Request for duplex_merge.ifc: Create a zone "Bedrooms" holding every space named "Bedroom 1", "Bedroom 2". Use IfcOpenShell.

First a look at what the model holds.

```python
import ifcopenshell

model = ifcopenshell.open("duplex_merge.ifc")
print(model.schema)
seen = {}
for space in model.by_type("IfcSpace"):
    seen[space.LongName] = seen.get(space.LongName, 0) + 1
for name, count in sorted(seen.items(), key=str):
    print(count, "x", name)
print("zones:", [z.Name for z in model.by_type("IfcZone")][:20])
```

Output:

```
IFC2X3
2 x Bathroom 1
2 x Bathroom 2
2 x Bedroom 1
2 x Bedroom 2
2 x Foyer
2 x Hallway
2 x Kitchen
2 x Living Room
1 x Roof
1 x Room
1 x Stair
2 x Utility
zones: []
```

```python
import ifcopenshell
import ifcopenshell.api.group
import ifcopenshell.api.root

model = ifcopenshell.open("duplex_merge.ifc")

names = {"Bedroom 1", "Bedroom 2"}
spaces = [s for s in model.by_type("IfcSpace") if s.LongName in names]

zone = ifcopenshell.api.root.create_entity(model, ifc_class="IfcZone", name="Bedrooms")
ifcopenshell.api.group.assign_group(model, products=spaces, group=zone)
print(len(spaces), "spaces in", zone.Name)

model.write("duplex_merge_v2.ifc")
```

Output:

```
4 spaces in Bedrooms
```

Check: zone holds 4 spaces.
